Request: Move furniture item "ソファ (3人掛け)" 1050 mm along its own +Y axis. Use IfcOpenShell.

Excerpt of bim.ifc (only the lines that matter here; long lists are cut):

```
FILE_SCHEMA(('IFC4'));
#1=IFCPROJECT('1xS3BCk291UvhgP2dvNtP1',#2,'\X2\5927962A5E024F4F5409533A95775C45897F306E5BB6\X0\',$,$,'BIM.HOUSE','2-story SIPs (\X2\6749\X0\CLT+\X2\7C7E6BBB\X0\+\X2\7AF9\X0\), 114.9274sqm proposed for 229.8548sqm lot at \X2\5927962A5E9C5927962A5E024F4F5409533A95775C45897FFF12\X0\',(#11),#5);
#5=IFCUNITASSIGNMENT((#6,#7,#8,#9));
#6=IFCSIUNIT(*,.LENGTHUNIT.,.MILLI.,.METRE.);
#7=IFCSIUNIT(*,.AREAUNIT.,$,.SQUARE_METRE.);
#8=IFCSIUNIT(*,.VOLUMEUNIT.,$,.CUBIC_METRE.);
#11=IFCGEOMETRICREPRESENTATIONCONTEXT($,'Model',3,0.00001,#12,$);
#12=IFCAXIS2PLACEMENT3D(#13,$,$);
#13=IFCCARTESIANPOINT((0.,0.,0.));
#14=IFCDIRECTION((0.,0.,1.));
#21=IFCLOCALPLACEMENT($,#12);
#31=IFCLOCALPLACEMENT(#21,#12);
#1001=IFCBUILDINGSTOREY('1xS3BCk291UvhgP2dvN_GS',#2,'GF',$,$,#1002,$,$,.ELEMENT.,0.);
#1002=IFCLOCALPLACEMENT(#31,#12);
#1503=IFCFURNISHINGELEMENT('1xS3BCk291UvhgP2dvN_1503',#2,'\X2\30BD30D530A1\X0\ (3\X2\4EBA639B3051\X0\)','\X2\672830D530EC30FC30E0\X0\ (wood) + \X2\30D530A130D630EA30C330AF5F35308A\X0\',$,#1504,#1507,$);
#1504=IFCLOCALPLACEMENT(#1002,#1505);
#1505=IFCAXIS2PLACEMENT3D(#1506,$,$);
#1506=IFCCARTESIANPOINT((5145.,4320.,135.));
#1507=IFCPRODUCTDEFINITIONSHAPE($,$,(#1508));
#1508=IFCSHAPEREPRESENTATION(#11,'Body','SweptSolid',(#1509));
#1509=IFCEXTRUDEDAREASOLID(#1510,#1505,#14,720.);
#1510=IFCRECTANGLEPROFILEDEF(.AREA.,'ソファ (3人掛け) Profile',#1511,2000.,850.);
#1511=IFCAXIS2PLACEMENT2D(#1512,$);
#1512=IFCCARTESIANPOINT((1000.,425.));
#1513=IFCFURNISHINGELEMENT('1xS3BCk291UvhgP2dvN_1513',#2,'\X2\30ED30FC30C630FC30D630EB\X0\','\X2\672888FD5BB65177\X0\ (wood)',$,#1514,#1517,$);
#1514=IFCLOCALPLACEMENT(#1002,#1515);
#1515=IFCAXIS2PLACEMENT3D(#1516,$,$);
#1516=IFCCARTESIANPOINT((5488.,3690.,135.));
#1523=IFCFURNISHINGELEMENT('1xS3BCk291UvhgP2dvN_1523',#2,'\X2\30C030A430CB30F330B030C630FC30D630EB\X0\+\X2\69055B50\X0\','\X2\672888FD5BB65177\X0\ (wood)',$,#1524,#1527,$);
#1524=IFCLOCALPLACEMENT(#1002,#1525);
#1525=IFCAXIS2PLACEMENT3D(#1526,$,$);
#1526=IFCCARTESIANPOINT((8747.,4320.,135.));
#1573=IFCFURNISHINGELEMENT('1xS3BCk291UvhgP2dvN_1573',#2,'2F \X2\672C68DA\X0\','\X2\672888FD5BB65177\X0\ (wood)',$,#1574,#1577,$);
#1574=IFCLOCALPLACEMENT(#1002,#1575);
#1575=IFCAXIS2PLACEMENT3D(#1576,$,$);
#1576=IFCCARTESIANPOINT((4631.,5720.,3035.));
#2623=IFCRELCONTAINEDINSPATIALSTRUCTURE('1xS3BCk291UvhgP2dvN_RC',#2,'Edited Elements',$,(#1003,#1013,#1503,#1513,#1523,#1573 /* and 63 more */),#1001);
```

```python
import ifcopenshell
import ifcopenshell.api.geometry
import ifcopenshell.util.placement
import ifcopenshell.util.unit

model = ifcopenshell.open("bim.ifc")
unit_scale = ifcopenshell.util.unit.calculate_unit_scale(model)

item = model.by_guid("1xS3BCk291UvhgP2dvN_1503")
matrix = ifcopenshell.util.placement.get_local_placement(item.ObjectPlacement)
matrix[:3, 3] += matrix[:3, 1] * 1.05 / unit_scale
ifcopenshell.api.geometry.edit_object_placement(model, product=item, matrix=matrix, is_si=False)

print(ifcopenshell.util.placement.get_local_placement(item.ObjectPlacement).round(3) + 0.0)

model.write("bim-out.ifc")
```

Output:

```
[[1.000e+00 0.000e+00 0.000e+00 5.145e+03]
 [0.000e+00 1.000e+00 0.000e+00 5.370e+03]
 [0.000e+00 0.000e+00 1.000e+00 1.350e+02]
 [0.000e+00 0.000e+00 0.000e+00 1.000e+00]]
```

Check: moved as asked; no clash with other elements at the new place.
